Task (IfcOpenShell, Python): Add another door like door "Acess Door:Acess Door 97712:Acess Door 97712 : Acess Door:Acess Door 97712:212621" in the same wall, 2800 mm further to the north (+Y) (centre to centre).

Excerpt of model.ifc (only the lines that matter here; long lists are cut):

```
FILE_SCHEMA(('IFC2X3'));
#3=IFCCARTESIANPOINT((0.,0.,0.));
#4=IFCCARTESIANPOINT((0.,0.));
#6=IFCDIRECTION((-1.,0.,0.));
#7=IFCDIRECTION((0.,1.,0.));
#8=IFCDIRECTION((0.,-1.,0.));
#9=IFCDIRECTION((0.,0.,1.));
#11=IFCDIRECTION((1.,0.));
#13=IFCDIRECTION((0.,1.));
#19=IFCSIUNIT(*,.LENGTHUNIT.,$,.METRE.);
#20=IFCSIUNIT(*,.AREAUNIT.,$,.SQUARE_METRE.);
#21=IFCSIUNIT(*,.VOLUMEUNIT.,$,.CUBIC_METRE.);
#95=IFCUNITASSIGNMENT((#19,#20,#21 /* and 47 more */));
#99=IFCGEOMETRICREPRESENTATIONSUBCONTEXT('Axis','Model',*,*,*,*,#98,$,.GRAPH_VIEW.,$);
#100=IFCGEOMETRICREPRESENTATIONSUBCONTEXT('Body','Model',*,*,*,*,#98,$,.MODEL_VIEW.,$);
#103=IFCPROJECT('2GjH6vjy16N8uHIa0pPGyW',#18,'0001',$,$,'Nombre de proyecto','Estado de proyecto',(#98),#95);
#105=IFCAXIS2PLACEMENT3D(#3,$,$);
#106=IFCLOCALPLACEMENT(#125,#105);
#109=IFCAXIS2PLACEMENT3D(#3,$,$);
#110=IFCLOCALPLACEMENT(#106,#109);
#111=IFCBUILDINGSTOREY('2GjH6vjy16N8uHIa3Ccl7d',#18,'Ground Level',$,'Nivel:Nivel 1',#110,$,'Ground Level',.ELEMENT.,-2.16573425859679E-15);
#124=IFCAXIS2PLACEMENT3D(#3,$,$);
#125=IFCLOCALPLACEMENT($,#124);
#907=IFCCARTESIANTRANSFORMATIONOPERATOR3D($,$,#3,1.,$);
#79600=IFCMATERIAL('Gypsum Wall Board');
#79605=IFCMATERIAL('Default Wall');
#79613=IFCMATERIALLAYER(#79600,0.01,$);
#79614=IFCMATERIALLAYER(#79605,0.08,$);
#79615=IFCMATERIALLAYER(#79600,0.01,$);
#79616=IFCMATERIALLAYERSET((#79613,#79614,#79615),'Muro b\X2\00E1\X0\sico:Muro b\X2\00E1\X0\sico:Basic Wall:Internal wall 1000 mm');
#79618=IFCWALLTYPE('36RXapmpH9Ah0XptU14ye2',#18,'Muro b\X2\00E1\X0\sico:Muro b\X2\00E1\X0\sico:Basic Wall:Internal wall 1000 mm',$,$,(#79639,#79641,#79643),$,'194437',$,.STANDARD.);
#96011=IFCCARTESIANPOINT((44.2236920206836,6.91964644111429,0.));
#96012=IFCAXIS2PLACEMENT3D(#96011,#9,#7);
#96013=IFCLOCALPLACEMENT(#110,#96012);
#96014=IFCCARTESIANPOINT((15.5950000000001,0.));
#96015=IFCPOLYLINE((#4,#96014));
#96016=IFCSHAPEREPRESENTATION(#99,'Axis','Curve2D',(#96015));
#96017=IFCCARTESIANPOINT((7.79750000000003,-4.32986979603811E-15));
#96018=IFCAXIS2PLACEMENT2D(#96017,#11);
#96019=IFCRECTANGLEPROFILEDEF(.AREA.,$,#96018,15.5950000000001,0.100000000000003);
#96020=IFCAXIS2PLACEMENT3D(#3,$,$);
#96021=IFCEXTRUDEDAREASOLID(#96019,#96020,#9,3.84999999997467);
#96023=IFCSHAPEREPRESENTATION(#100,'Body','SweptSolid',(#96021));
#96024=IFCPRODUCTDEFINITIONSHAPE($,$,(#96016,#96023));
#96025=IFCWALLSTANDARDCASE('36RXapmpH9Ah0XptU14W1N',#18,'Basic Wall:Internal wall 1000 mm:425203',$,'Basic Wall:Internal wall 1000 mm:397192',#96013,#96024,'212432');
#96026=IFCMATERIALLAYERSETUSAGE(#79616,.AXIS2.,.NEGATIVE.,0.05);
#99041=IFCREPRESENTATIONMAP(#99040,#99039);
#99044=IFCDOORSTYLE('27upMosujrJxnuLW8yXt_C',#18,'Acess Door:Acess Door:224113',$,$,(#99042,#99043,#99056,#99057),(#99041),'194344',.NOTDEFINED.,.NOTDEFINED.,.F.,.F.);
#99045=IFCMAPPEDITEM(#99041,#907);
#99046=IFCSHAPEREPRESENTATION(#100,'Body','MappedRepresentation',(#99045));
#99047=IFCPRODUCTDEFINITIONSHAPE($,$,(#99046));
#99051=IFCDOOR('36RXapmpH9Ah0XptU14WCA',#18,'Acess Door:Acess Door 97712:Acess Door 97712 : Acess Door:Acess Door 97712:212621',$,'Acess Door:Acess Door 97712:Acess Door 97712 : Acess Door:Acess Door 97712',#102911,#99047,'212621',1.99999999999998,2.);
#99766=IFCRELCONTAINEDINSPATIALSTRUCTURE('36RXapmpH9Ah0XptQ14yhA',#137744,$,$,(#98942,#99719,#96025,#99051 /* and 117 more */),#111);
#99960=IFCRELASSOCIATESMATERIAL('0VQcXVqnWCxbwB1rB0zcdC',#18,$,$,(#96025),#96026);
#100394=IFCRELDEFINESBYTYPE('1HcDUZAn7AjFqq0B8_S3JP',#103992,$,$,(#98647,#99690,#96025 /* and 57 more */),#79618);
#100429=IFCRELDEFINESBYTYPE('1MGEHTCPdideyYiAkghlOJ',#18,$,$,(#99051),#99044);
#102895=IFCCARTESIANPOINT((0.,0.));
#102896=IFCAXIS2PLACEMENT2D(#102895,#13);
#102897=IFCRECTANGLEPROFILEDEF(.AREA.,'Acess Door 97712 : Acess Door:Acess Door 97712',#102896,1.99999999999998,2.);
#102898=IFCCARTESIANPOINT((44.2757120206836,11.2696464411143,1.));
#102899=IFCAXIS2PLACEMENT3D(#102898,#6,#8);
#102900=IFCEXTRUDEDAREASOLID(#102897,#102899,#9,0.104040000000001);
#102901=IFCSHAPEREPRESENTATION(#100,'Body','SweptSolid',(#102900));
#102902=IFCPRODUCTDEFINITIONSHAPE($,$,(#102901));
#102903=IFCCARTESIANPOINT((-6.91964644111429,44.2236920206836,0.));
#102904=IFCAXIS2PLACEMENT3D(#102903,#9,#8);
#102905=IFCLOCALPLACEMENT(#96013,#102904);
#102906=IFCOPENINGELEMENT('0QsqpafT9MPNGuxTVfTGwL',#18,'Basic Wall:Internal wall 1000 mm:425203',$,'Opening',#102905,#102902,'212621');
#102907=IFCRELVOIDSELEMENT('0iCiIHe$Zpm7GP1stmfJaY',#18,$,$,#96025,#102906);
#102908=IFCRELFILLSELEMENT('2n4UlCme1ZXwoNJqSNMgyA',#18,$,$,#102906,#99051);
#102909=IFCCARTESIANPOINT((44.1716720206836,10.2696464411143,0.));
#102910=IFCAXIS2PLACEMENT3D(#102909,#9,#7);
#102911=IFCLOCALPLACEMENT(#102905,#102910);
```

```python
import ifcopenshell
import ifcopenshell.api.feature
import ifcopenshell.api.geometry
import ifcopenshell.api.root
import ifcopenshell.geom
import ifcopenshell.util.element
import ifcopenshell.util.placement
import ifcopenshell.util.shape

model = ifcopenshell.open("model.ifc")
settings = ifcopenshell.geom.settings()


def volume(element):
    """Net volume in cubic metres, openings subtracted."""
    shape = ifcopenshell.geom.create_shape(settings, element)
    return ifcopenshell.util.shape.get_volume(shape.geometry)


def reuse_history(source, copy):
    """copy_class also copies each property set's owner history, people and application; keep the originals."""
    for rel in copy.IsDefinedBy:
        if rel.is_a("IfcRelDefinesByProperties") and (history := rel.RelatingPropertyDefinition.OwnerHistory):
            rel.RelatingPropertyDefinition.OwnerHistory = source.OwnerHistory
            ifcopenshell.util.element.remove_deep2(model, history)


door = model.by_guid("36RXapmpH9Ah0XptU14WCA")
opening = door.FillsVoids[0].RelatingOpeningElement
wall = opening.VoidsElements[0].RelatingBuildingElement
before = volume(wall)
shift = ifcopenshell.util.placement.get_local_placement(wall.ObjectPlacement)[:3, 0] * 2.8

# copy_class copies the void relationship, type, container and properties, but no geometry.
new_opening = ifcopenshell.api.root.copy_class(model, product=opening)
new_opening.Representation = ifcopenshell.util.element.copy_deep(
    model, opening.Representation, exclude=["IfcGeometricRepresentationContext", "IfcRepresentationMap"]
)
new_opening.Name = "Basic Wall:Internal wall 1000 mm"
new_opening.Tag = None
new_door = ifcopenshell.api.root.copy_class(model, product=door)
new_door.Representation = ifcopenshell.util.element.copy_deep(
    model, door.Representation, exclude=["IfcGeometricRepresentationContext", "IfcRepresentationMap"]
)
new_door.Name = "Acess Door:Acess Door 97712:Acess Door 97712 : Acess Door:Acess Door 97712"
new_door.Tag = None
reuse_history(door, new_door)
fills = ifcopenshell.api.feature.add_filling(model, opening=new_opening, element=new_door)
fills.OwnerHistory = new_door.OwnerHistory  # required in IFC2X3

for old, new in ((opening, new_opening), (door, new_door)):
    matrix = ifcopenshell.util.placement.get_local_placement(old.ObjectPlacement)
    matrix[:3, 3] += shift
    ifcopenshell.api.geometry.edit_object_placement(model, product=new, matrix=matrix, is_si=False)

after = volume(wall)

print(f"wall volume {before:.3f} -> {after:.3f} m3")

model.write("model_rev.ifc")
```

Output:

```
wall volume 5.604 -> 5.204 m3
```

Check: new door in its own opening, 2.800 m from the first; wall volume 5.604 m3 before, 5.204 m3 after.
